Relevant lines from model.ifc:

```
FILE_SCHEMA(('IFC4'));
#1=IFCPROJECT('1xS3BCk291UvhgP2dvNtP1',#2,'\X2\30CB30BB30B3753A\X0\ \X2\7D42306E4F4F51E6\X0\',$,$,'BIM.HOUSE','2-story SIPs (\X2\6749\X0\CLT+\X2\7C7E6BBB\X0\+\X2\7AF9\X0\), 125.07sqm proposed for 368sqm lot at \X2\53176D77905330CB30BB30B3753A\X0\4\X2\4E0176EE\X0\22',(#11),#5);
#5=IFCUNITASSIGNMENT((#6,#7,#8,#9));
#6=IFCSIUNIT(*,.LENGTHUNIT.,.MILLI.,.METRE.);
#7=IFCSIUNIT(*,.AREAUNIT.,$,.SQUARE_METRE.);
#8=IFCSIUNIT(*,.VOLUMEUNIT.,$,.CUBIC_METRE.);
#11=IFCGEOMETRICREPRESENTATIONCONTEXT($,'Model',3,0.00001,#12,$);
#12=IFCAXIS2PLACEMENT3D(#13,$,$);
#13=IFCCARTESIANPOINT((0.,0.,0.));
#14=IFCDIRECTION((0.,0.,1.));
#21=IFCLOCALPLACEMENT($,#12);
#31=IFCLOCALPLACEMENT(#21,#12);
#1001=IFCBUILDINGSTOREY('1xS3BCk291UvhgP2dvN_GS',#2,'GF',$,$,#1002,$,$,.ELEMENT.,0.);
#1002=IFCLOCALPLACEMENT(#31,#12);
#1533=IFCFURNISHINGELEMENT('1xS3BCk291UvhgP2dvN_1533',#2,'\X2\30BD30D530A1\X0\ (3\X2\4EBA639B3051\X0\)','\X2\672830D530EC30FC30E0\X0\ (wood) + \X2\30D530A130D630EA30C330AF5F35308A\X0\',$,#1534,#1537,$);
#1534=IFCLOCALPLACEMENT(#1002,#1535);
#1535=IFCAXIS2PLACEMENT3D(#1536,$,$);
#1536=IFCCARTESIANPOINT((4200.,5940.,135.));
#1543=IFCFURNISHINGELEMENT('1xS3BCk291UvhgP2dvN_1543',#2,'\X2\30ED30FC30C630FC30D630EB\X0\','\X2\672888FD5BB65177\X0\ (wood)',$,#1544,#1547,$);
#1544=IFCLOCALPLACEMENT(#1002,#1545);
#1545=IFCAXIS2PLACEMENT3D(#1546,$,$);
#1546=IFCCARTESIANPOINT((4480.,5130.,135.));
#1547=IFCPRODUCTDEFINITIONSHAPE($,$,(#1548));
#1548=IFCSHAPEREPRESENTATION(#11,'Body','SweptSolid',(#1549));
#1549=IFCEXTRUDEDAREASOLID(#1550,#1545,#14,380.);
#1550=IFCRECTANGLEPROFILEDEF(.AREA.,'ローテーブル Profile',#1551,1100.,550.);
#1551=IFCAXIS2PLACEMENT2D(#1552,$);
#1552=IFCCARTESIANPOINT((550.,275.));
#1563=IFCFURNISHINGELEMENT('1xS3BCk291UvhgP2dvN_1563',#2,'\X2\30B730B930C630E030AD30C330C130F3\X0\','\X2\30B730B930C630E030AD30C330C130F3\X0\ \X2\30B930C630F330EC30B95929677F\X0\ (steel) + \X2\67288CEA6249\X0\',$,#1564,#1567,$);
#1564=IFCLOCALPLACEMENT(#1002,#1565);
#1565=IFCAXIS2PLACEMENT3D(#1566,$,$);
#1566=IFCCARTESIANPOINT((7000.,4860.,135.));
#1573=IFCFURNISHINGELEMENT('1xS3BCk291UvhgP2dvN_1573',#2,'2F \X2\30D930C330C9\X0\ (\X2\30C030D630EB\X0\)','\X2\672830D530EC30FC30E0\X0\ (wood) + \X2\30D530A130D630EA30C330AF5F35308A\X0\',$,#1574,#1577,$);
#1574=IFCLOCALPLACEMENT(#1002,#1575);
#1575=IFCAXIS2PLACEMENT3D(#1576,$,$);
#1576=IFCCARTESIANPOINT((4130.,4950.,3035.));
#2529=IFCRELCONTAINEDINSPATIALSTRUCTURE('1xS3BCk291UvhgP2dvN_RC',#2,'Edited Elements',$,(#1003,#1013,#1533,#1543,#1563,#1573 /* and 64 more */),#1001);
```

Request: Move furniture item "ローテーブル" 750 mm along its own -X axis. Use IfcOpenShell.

```python
import ifcopenshell
import ifcopenshell.api.geometry
import ifcopenshell.util.placement
import ifcopenshell.util.unit

model = ifcopenshell.open("model.ifc")
unit_scale = ifcopenshell.util.unit.calculate_unit_scale(model)

item = model.by_id(1543)
matrix = ifcopenshell.util.placement.get_local_placement(item.ObjectPlacement)
matrix[:3, 3] -= matrix[:3, 0] * 0.75 / unit_scale
ifcopenshell.api.geometry.edit_object_placement(model, product=item, matrix=matrix, is_si=False)

print(ifcopenshell.util.placement.get_local_placement(item.ObjectPlacement).round(3) + 0.0)

model.write("model_v2.ifc")
```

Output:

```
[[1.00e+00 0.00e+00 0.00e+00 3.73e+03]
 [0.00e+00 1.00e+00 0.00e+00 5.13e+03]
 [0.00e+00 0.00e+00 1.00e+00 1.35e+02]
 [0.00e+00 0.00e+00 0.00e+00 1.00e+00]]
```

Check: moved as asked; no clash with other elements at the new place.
